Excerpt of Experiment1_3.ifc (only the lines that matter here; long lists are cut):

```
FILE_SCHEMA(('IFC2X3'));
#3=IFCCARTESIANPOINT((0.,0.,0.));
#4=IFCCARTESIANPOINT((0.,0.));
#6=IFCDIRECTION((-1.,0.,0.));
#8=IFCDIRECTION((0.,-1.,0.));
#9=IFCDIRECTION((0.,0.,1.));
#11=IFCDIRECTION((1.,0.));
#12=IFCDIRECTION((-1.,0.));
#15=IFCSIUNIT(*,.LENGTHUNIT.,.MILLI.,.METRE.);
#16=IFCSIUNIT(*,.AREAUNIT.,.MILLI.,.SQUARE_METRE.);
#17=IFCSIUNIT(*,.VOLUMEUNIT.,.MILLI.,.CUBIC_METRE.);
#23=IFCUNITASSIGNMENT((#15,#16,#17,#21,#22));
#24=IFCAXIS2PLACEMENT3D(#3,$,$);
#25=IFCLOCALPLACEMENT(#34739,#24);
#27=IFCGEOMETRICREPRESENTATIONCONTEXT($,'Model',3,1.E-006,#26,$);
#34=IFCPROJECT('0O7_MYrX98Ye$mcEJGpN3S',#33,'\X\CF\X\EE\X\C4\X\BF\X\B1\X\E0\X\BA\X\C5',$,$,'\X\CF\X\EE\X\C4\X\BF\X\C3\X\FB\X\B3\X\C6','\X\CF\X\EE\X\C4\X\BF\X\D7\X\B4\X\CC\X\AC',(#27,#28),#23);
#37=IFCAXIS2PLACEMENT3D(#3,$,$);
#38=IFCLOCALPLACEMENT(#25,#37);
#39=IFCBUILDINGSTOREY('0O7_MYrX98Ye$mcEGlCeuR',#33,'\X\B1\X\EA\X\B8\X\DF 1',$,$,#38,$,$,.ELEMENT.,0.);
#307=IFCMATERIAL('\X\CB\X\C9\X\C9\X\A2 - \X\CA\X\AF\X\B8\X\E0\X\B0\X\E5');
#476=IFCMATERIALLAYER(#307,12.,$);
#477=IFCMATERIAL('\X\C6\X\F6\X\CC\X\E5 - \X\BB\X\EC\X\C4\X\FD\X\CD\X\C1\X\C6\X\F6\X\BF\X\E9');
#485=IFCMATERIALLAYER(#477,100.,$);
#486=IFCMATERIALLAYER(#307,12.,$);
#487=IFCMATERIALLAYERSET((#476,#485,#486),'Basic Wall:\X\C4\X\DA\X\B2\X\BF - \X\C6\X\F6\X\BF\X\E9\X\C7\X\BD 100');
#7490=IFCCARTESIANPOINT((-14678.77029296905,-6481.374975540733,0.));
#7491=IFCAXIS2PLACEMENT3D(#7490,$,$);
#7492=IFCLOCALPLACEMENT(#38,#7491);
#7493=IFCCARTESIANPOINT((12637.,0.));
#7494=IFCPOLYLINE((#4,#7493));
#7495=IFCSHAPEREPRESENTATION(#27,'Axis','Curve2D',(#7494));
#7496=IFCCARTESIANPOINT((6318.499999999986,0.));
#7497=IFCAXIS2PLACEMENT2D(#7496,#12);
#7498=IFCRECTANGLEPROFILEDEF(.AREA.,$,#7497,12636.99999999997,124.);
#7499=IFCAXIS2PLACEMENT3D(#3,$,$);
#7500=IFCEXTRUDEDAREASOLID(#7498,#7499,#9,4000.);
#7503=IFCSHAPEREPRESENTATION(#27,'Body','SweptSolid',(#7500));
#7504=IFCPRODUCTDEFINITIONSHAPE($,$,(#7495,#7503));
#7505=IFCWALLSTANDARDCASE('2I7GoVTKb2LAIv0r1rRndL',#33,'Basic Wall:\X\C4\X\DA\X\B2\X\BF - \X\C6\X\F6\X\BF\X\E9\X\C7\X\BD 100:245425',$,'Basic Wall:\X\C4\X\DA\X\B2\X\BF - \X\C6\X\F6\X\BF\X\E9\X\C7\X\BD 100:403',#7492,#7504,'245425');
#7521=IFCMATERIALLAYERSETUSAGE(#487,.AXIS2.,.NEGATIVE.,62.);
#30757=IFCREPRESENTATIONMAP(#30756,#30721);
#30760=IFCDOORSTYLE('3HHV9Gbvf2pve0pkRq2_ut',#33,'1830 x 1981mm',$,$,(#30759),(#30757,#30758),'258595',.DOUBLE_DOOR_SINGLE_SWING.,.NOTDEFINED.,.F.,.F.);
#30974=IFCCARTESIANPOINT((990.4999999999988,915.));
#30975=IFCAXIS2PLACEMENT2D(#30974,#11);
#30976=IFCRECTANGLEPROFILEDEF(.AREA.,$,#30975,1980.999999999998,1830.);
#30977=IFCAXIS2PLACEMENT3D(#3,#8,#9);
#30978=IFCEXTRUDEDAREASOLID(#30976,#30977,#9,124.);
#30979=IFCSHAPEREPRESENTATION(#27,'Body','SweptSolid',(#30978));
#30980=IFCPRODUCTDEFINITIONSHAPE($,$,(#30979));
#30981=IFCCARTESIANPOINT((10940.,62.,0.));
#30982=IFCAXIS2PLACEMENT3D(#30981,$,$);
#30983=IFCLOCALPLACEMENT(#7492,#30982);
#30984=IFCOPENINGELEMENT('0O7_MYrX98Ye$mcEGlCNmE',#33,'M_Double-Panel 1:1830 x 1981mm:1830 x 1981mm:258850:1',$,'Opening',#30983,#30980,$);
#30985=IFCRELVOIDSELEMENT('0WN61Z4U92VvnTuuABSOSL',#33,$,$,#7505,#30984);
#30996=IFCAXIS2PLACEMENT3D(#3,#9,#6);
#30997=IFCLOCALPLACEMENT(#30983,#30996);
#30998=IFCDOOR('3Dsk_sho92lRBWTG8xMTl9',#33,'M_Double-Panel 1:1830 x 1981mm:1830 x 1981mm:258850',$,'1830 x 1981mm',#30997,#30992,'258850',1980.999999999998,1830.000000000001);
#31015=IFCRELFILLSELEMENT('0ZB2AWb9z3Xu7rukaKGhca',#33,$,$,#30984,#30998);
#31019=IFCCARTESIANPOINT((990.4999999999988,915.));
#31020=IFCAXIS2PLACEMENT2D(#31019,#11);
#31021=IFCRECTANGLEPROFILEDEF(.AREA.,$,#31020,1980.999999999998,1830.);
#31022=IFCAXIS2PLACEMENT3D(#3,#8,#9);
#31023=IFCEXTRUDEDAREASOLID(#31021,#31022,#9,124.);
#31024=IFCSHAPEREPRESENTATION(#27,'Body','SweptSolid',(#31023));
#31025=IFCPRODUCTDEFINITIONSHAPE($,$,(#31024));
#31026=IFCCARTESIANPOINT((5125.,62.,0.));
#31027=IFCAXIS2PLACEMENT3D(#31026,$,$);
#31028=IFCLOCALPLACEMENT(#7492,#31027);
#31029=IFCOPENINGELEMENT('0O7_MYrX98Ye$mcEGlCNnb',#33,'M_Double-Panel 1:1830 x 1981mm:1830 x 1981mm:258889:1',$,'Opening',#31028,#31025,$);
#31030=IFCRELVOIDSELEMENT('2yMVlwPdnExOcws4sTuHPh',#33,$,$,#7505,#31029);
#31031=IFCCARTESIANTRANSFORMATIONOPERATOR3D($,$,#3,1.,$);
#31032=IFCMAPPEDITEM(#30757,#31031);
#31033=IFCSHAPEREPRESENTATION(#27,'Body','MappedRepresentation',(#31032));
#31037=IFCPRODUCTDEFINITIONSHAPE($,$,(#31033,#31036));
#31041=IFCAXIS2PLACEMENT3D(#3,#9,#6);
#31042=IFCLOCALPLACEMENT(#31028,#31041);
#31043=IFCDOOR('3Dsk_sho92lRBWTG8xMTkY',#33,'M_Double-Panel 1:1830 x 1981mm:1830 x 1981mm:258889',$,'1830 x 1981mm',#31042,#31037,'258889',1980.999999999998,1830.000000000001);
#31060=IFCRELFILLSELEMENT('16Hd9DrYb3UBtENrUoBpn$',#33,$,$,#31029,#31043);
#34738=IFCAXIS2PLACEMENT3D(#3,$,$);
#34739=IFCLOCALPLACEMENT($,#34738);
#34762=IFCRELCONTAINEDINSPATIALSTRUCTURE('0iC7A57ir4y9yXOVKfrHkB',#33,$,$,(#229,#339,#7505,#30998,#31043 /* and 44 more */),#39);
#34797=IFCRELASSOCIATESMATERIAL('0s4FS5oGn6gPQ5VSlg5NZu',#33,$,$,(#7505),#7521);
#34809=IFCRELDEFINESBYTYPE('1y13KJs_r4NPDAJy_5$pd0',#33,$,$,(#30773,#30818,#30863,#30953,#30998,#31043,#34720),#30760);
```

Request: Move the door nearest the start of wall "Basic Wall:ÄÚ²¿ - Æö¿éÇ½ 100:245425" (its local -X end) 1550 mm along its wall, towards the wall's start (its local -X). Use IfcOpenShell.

```python
import ifcopenshell
import ifcopenshell.api.geometry
import ifcopenshell.util.placement
import ifcopenshell.util.unit

model = ifcopenshell.open("Experiment1_3.ifc")
unit_scale = ifcopenshell.util.unit.calculate_unit_scale(model)

door = model.by_guid("3Dsk_sho92lRBWTG8xMTkY")
opening = door.FillsVoids[0].RelatingOpeningElement
wall = opening.VoidsElements[0].RelatingBuildingElement

wall_matrix = ifcopenshell.util.placement.get_local_placement(wall.ObjectPlacement)
shift = wall_matrix[:3, 0] * -1.55 / unit_scale
before = ifcopenshell.util.placement.get_local_placement(door.ObjectPlacement)[:3, 3].copy()

# The door is placed relative to its opening, so it follows when the opening moves.
matrix = ifcopenshell.util.placement.get_local_placement(opening.ObjectPlacement)
matrix[:3, 3] += shift
ifcopenshell.api.geometry.edit_object_placement(
    model, product=opening, matrix=matrix, is_si=False, should_transform_children=True
)

after = ifcopenshell.util.placement.get_local_placement(door.ObjectPlacement)[:3, 3]
print("door moved by", (after - before).round(3) + 0.0)

model.write("Experiment1_3_updated.ifc")
```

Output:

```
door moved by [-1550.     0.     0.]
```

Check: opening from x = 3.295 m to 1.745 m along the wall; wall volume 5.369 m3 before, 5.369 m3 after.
